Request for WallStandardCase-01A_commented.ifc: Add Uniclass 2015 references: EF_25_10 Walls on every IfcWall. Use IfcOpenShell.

First a look at what the model holds.

```python
import ifcopenshell

model = ifcopenshell.open("WallStandardCase-01A_commented.ifc")
print(model.schema)
print("classifications:", [c.Name for c in model.by_type("IfcClassification")])
for ifc_class in ("IfcDoor", "IfcRoof", "IfcStair", "IfcWall", "IfcWindow"):
    print(ifc_class, len(model.by_type(ifc_class)))
```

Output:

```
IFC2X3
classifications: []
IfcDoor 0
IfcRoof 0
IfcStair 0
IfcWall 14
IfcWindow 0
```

```python
import ifcopenshell
import ifcopenshell.api.classification

model = ifcopenshell.open("WallStandardCase-01A_commented.ifc")

# IFC2X3 requires Source and Edition and has no link from the project to the system.
system = model.create_entity("IfcClassification", Source="NBS", Edition="2015", Name="Uniclass 2015")

codes = {
    "IfcWall": ("EF_25_10", "Walls"),
}
for ifc_class, (code, name) in codes.items():
    products = model.by_type(ifc_class)
    ifcopenshell.api.classification.add_reference(
        model, products=products, classification=system, identification=code, name=name
    )
    print(code, len(products))

model.write("WallStandardCase-01A_commented_updated.ifc")
```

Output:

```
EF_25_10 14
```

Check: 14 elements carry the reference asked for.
